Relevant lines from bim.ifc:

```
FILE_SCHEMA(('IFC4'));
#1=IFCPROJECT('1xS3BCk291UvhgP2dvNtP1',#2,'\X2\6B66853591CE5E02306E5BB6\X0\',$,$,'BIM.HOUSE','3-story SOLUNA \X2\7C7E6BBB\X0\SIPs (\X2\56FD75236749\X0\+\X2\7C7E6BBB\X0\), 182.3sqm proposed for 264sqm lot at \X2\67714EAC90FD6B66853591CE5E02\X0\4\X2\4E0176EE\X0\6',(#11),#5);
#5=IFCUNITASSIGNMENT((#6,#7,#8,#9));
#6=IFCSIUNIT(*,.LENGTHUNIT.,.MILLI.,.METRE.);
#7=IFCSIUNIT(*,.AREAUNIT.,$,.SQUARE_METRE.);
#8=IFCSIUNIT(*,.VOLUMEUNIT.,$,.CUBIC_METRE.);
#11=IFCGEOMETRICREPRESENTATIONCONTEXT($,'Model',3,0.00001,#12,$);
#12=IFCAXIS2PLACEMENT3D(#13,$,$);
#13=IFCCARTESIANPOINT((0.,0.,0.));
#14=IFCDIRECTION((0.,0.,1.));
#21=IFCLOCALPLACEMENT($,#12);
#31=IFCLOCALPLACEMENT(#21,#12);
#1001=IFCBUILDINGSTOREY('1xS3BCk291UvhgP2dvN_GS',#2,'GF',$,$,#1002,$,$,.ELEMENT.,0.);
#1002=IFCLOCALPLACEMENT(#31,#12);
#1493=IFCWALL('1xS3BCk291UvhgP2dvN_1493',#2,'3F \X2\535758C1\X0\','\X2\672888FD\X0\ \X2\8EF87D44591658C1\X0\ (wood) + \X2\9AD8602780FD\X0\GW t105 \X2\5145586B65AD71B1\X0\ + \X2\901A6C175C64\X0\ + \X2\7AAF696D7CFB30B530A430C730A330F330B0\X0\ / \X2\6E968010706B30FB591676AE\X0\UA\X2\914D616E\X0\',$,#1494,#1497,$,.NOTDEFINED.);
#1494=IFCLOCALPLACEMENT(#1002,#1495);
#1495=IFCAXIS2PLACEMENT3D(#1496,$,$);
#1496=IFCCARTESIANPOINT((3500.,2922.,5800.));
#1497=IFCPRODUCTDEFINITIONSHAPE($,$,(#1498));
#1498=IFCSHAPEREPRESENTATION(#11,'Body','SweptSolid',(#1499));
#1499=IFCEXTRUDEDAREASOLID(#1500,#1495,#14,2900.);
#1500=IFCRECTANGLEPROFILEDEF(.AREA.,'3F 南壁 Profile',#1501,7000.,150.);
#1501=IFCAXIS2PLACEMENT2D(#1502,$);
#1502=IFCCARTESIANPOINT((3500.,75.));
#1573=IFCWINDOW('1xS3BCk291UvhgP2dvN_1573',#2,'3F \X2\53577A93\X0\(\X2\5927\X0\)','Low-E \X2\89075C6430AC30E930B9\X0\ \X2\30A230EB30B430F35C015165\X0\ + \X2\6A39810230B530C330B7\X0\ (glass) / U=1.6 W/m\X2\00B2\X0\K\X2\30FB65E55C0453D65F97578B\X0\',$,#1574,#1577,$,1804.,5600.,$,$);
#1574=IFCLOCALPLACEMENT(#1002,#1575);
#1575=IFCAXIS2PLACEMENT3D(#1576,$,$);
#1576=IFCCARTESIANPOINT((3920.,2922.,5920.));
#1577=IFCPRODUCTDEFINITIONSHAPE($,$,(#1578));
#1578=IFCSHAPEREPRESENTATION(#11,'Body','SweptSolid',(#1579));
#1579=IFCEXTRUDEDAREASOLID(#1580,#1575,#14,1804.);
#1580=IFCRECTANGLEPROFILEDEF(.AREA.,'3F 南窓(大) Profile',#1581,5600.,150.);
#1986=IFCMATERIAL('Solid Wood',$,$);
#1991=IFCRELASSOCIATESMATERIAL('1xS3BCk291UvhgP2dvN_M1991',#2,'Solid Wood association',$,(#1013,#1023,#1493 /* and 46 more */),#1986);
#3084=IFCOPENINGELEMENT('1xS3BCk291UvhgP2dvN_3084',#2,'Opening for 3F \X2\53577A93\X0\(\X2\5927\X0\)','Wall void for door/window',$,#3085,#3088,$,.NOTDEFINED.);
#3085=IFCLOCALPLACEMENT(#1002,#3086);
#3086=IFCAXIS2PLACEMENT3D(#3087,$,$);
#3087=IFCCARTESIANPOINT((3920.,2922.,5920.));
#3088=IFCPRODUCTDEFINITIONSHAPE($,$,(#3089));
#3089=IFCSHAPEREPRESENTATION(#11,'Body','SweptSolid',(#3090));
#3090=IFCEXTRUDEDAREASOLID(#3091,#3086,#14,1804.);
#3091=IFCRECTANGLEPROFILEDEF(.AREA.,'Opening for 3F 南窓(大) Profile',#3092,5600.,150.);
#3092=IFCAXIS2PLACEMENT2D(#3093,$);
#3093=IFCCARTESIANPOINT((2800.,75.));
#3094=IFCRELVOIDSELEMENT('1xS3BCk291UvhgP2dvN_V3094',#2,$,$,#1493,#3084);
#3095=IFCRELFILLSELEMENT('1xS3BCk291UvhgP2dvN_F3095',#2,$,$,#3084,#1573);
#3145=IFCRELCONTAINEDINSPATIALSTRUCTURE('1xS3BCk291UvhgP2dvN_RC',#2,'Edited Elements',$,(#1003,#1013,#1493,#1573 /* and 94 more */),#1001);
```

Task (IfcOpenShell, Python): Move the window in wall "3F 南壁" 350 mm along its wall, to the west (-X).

```python
import ifcopenshell
import ifcopenshell.api.geometry
import ifcopenshell.util.placement
import ifcopenshell.util.unit

model = ifcopenshell.open("bim.ifc")
unit_scale = ifcopenshell.util.unit.calculate_unit_scale(model)

window = model.by_guid("1xS3BCk291UvhgP2dvN_1573")
opening = window.FillsVoids[0].RelatingOpeningElement
wall = opening.VoidsElements[0].RelatingBuildingElement

wall_matrix = ifcopenshell.util.placement.get_local_placement(wall.ObjectPlacement)
shift = wall_matrix[:3, 0] * -0.35 / unit_scale
before = ifcopenshell.util.placement.get_local_placement(window.ObjectPlacement)[:3, 3].copy()

# The window is not placed relative to its opening, so move both.
for product in (opening, window):
    matrix = ifcopenshell.util.placement.get_local_placement(product.ObjectPlacement)
    matrix[:3, 3] += shift
    ifcopenshell.api.geometry.edit_object_placement(model, product=product, matrix=matrix, is_si=False)

after = ifcopenshell.util.placement.get_local_placement(window.ObjectPlacement)[:3, 3]
print("window moved by", (after - before).round(3) + 0.0)

model.write("bim_edited.ifc")
```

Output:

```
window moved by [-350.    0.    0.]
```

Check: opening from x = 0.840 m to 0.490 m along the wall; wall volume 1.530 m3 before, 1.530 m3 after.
